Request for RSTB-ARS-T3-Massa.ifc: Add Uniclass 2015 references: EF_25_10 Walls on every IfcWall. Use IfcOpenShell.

First a look at what the model holds.

```python
import ifcopenshell

model = ifcopenshell.open("RSTB-ARS-T3-Massa.ifc")
print(model.schema)
print("classifications:", [c.Name for c in model.by_type("IfcClassification")])
for ifc_class in ("IfcDoor", "IfcRoof", "IfcStair", "IfcWall", "IfcWindow"):
    print(ifc_class, len(model.by_type(ifc_class)))
```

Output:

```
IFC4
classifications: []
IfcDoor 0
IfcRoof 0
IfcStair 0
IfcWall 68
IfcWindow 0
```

```python
import ifcopenshell
import ifcopenshell.api.classification

model = ifcopenshell.open("RSTB-ARS-T3-Massa.ifc")

system = ifcopenshell.api.classification.add_classification(model, classification="Uniclass 2015")

codes = {
    "IfcWall": ("EF_25_10", "Walls"),
}
for ifc_class, (code, name) in codes.items():
    products = model.by_type(ifc_class)
    ifcopenshell.api.classification.add_reference(
        model, products=products, classification=system, identification=code, name=name
    )
    print(code, len(products))

model.write("RSTB-ARS-T3-Massa_v2.ifc")
```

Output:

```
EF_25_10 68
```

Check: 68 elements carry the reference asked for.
